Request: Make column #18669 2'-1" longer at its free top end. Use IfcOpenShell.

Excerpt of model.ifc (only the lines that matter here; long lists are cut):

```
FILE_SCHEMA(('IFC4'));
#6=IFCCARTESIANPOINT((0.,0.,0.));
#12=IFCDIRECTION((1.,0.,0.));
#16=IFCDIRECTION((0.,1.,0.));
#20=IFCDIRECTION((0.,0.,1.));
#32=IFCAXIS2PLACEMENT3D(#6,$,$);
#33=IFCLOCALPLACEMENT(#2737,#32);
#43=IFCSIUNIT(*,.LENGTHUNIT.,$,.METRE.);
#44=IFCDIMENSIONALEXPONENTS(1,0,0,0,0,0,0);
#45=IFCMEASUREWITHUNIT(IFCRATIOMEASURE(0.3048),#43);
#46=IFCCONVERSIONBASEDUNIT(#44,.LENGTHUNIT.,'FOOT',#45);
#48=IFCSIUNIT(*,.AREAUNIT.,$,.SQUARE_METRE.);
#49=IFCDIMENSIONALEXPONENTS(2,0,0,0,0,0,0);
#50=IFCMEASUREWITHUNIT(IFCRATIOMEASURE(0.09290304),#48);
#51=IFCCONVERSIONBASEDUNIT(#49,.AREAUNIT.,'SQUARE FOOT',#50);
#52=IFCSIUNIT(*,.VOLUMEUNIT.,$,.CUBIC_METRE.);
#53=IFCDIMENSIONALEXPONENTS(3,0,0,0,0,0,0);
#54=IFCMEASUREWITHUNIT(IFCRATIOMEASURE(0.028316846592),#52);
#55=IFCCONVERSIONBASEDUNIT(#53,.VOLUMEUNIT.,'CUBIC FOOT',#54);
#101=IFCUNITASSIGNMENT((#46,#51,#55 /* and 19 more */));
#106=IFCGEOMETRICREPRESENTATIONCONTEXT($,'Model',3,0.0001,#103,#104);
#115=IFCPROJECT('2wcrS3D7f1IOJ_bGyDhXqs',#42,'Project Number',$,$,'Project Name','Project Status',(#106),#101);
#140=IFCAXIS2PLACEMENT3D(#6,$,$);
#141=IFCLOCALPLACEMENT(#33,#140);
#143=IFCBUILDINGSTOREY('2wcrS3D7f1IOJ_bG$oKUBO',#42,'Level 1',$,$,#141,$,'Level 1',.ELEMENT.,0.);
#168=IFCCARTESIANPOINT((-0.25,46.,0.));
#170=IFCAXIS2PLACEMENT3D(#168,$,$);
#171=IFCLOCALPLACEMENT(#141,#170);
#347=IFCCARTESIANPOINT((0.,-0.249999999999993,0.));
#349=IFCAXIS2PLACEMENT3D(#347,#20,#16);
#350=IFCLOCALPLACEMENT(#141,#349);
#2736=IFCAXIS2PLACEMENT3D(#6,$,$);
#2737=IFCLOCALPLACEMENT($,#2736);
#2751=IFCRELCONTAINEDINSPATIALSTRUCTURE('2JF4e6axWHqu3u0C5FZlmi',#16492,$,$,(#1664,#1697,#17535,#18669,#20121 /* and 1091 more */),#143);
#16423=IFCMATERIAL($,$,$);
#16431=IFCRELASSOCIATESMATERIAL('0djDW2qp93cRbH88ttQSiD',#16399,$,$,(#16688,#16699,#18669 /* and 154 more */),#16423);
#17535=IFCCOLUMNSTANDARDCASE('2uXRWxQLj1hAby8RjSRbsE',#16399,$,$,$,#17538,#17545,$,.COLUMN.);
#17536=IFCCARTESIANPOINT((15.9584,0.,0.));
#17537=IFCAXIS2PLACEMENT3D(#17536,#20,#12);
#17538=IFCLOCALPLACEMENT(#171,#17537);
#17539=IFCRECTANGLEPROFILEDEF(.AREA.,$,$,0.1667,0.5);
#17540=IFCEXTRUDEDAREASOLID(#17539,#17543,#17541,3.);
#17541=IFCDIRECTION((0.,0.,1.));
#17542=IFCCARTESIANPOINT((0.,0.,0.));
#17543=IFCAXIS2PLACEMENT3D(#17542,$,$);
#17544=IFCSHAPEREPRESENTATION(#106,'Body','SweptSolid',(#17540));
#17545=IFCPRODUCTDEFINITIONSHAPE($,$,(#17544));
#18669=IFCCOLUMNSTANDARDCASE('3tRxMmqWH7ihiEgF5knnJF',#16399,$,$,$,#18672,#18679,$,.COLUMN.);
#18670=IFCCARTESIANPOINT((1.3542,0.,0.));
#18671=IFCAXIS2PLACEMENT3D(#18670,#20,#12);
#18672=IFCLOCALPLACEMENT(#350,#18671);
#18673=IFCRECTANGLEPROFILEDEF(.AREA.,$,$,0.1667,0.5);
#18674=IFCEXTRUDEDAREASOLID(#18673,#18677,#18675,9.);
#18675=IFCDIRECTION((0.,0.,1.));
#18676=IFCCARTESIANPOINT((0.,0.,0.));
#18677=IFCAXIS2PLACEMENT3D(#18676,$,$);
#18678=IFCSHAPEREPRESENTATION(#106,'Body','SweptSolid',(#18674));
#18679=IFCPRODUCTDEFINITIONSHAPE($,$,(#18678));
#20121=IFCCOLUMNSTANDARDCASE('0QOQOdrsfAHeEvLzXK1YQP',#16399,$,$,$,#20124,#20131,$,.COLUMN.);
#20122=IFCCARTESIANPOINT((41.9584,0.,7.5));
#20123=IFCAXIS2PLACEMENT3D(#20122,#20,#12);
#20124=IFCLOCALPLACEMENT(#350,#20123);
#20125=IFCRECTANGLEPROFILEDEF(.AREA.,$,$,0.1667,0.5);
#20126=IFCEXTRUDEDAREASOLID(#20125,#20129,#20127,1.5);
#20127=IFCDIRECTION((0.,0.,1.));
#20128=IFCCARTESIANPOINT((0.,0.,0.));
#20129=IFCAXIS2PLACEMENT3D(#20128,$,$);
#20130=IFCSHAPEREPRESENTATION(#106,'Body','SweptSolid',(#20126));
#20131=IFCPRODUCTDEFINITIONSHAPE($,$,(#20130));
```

```python
import ifcopenshell
import ifcopenshell.util.unit

model = ifcopenshell.open("model.ifc")
unit_scale = ifcopenshell.util.unit.calculate_unit_scale(model)

member = model.by_guid("3tRxMmqWH7ihiEgF5knnJF")
change = 25 * 0.0254 / unit_scale

# The extrusion runs towards the end named, so only its depth changes.
body = next(r for r in member.Representation.Representations if r.RepresentationIdentifier == "Body")
solid = body.Items[0]
old_length = solid.Depth
solid.Depth += change

print(f"length {old_length:g} -> {solid.Depth:g}")

model.write("model_updated.ifc")
```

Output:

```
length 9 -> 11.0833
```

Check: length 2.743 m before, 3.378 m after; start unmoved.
